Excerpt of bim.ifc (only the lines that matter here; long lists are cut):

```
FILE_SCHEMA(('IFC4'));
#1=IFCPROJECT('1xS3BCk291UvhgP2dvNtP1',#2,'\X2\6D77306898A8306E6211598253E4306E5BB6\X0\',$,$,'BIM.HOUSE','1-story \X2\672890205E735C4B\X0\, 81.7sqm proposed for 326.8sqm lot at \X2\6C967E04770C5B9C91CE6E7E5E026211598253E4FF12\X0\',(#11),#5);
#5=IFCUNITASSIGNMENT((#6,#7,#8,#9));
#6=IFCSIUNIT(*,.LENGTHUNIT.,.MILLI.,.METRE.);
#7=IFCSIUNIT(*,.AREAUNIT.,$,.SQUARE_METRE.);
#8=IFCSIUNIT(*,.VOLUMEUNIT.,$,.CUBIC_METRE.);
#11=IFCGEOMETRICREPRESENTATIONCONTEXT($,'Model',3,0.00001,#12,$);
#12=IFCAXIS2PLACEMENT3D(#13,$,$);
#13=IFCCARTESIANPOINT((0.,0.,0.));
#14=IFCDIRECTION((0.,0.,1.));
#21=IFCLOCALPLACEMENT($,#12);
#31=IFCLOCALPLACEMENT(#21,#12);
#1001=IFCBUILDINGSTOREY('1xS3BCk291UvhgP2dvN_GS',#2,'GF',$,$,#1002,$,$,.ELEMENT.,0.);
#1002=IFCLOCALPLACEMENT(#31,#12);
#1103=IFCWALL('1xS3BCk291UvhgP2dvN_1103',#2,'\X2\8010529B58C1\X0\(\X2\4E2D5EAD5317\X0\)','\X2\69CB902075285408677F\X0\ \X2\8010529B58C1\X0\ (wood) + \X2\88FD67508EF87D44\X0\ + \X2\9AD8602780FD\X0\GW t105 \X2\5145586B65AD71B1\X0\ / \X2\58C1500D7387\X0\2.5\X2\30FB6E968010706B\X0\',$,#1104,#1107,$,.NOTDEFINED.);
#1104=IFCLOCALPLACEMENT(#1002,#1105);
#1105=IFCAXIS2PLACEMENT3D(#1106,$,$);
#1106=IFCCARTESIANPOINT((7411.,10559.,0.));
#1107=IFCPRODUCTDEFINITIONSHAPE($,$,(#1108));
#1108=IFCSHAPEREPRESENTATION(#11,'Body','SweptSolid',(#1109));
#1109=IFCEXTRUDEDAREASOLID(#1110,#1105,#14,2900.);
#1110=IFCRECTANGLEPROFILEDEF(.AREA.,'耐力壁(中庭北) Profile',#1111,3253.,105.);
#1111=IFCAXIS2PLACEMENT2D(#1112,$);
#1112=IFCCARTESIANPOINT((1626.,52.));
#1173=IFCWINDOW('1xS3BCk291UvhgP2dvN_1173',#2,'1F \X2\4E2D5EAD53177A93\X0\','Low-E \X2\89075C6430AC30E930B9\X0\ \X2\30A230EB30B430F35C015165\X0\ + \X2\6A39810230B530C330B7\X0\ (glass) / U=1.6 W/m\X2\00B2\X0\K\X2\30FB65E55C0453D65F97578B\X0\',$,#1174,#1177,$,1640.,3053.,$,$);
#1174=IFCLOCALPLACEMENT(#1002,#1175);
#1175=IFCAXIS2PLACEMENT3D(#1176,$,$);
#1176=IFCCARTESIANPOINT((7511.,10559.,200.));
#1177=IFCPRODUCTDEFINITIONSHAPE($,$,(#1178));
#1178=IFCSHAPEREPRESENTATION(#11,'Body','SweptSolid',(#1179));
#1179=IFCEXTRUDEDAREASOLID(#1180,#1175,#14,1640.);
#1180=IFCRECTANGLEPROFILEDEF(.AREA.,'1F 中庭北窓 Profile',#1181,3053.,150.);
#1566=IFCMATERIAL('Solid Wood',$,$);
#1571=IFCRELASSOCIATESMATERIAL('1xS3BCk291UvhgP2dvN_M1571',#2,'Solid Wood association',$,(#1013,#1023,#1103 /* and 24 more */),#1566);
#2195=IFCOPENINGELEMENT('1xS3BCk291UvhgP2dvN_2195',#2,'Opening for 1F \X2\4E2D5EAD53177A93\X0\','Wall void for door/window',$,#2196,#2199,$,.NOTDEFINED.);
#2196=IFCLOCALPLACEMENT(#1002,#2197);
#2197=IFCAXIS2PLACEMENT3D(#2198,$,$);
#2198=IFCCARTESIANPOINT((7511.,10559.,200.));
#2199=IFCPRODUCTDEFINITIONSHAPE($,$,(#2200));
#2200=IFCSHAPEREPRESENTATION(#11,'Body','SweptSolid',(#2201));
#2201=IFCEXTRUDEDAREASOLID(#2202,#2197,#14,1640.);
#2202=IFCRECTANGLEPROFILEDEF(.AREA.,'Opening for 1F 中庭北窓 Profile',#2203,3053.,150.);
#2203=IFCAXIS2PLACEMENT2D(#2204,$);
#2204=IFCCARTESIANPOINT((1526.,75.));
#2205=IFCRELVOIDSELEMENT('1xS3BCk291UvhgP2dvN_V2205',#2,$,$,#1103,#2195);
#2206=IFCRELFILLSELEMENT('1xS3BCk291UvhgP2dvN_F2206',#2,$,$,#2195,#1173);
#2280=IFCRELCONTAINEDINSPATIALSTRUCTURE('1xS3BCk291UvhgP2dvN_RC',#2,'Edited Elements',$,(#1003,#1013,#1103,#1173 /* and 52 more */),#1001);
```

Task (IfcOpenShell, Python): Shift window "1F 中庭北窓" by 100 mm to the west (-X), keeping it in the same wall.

```python
import ifcopenshell
import ifcopenshell.api.geometry
import ifcopenshell.util.placement

model = ifcopenshell.open("bim.ifc")

window = model.by_guid("1xS3BCk291UvhgP2dvN_1173")
opening = window.FillsVoids[0].RelatingOpeningElement
wall = opening.VoidsElements[0].RelatingBuildingElement

wall_matrix = ifcopenshell.util.placement.get_local_placement(wall.ObjectPlacement)
shift = wall_matrix[:3, 0] * -100.0
before = ifcopenshell.util.placement.get_local_placement(window.ObjectPlacement)[:3, 3].copy()

# The window is not placed relative to its opening, so move both.
for product in (opening, window):
    matrix = ifcopenshell.util.placement.get_local_placement(product.ObjectPlacement)
    matrix[:3, 3] += shift
    ifcopenshell.api.geometry.edit_object_placement(model, product=product, matrix=matrix, is_si=False)

after = ifcopenshell.util.placement.get_local_placement(window.ObjectPlacement)[:3, 3]
print("window moved by", (after - before).round(3) + 0.0)

model.write("bim_v2.ifc")
```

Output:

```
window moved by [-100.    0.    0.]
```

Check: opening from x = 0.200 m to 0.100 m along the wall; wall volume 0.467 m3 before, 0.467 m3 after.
